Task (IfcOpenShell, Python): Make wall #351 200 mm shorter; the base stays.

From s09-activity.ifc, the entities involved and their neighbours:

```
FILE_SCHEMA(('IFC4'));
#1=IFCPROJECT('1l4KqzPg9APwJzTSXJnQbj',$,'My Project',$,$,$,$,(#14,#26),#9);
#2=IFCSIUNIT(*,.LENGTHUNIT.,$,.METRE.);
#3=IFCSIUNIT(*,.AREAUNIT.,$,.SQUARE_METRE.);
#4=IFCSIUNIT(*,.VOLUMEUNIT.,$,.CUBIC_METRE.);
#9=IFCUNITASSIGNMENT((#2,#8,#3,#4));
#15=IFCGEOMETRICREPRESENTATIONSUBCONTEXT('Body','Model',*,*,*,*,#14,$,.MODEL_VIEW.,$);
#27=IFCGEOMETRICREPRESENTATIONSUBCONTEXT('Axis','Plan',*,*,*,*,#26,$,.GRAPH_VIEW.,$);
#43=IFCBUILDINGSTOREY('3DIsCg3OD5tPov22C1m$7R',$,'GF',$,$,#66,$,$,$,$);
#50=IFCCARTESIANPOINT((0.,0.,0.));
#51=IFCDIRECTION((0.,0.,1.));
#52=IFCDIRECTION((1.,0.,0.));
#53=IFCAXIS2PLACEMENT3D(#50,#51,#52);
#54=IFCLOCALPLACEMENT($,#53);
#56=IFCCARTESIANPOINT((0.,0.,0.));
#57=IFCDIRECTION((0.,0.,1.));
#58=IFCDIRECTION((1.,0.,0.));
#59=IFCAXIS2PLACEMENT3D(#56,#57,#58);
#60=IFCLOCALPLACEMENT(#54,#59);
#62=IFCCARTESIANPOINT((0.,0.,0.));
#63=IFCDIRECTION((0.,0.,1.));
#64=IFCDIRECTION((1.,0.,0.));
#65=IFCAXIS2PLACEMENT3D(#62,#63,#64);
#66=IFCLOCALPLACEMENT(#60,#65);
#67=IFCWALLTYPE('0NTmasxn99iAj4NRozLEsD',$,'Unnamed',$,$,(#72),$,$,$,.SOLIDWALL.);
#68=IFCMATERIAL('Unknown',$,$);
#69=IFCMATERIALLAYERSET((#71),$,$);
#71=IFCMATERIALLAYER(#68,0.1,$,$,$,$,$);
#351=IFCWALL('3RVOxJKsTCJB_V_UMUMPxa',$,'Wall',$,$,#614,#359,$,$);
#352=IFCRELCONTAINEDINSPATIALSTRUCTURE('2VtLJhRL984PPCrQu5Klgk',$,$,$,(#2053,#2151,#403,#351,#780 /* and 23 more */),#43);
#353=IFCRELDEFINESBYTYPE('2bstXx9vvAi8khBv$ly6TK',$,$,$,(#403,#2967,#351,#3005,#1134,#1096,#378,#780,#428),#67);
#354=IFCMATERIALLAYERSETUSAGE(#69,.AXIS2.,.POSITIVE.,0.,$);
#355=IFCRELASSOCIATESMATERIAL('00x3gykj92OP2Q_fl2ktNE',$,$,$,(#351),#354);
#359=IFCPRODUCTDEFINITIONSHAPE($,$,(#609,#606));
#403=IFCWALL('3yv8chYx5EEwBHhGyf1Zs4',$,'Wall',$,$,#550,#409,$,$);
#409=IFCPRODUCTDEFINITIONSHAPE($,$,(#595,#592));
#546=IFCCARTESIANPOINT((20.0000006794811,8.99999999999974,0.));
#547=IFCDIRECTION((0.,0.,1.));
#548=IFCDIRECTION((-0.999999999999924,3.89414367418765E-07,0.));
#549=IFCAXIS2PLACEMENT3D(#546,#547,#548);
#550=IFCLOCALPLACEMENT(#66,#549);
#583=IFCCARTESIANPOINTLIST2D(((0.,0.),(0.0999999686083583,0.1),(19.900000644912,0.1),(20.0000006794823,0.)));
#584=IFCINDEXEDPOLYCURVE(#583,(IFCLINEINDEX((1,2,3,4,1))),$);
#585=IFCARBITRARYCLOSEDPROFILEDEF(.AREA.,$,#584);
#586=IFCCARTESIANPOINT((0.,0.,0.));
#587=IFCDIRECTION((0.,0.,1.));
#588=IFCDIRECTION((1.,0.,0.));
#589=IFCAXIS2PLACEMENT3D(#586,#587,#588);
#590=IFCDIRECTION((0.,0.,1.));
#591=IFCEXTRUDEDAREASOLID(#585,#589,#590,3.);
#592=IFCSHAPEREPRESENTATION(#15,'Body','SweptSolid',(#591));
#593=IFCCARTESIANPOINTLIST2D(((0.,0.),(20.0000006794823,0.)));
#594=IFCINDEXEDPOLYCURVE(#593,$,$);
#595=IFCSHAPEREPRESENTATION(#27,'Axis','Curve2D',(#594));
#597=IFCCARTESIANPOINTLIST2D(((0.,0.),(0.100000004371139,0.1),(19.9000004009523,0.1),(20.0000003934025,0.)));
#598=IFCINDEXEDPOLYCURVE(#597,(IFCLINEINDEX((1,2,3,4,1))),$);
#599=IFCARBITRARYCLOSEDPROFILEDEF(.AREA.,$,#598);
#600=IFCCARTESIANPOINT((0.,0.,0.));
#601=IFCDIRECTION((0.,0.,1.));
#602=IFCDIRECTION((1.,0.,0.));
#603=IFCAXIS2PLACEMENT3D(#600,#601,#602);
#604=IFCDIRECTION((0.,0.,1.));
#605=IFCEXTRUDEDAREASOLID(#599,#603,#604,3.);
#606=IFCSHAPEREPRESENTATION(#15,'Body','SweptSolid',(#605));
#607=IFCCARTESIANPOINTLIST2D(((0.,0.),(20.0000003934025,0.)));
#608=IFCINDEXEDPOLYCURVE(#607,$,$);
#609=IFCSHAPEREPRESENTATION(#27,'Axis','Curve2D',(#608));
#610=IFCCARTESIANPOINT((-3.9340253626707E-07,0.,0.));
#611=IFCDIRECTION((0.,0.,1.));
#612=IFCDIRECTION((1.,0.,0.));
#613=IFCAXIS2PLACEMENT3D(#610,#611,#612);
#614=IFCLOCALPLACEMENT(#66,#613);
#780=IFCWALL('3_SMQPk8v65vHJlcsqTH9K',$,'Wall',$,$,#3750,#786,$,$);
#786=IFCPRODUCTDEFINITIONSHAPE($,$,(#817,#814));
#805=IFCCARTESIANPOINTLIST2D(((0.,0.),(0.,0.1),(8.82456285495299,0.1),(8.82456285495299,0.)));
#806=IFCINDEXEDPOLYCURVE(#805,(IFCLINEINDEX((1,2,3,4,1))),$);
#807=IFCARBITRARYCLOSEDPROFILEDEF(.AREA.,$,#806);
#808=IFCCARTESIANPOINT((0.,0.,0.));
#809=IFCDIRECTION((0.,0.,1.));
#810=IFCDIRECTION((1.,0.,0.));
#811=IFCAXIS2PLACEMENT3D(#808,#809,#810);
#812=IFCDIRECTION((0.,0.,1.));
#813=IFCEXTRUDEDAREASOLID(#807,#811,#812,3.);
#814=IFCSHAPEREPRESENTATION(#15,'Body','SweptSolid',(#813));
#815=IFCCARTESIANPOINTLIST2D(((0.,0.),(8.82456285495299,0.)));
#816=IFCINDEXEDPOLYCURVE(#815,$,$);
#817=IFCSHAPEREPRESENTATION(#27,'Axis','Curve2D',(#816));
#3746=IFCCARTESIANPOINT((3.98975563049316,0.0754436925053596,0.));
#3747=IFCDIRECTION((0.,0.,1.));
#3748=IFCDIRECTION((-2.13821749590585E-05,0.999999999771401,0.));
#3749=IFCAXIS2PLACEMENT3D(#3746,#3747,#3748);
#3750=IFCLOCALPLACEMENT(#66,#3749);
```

```python
import ifcopenshell
import ifcopenshell.geom
import ifcopenshell.util.representation
import ifcopenshell.util.shape
import ifcopenshell.util.unit

model = ifcopenshell.open("s09-activity.ifc")
unit_scale = ifcopenshell.util.unit.calculate_unit_scale(model)
settings = ifcopenshell.geom.settings()


def volume(element):
    """Net volume in cubic metres, openings subtracted."""
    shape = ifcopenshell.geom.create_shape(settings, element)
    return ifcopenshell.util.shape.get_volume(shape.geometry)


wall = model.by_guid("3RVOxJKsTCJB_V_UMUMPxa")
before = volume(wall)

body = ifcopenshell.util.representation.get_representation(wall, "Model", "Body")
solid = body.Items[0]
old_height = solid.Depth
solid.Depth -= 0.2 / unit_scale
after = volume(wall)

print(f"height {old_height:g} -> {solid.Depth:g}, volume {before:.3f} -> {after:.3f} m3")

model.write("s09-activity-out.ifc")
```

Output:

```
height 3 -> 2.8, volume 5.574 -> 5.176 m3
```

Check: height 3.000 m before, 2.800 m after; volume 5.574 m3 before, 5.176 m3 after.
